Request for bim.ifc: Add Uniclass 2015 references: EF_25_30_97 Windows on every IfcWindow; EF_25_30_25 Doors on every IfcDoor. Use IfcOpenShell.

First a look at what the model holds.

```python
import ifcopenshell

model = ifcopenshell.open("bim.ifc")
print(model.schema)
print("classifications:", [c.Name for c in model.by_type("IfcClassification")])
for ifc_class in ("IfcDoor", "IfcRoof", "IfcStair", "IfcWall", "IfcWindow"):
    print(ifc_class, len(model.by_type(ifc_class)))
```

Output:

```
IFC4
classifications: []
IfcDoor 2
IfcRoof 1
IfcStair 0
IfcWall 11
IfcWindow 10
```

```python
import ifcopenshell
import ifcopenshell.api.classification

model = ifcopenshell.open("bim.ifc")

system = ifcopenshell.api.classification.add_classification(model, classification="Uniclass 2015")

codes = {
    "IfcWindow": ("EF_25_30_97", "Windows"),
    "IfcDoor": ("EF_25_30_25", "Doors"),
}
for ifc_class, (code, name) in codes.items():
    products = model.by_type(ifc_class)
    ifcopenshell.api.classification.add_reference(
        model, products=products, classification=system, identification=code, name=name
    )
    print(code, len(products))

model.write("bim-out.ifc")
```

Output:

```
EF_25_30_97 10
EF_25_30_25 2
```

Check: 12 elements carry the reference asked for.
